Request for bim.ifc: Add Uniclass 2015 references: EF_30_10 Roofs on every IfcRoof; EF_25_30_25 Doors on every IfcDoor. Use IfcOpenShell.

First a look at what the model holds.

```python
import ifcopenshell

model = ifcopenshell.open("bim.ifc")
print(model.schema)
print("classifications:", [c.Name for c in model.by_type("IfcClassification")])
for ifc_class in ("IfcDoor", "IfcRoof", "IfcStair", "IfcWall", "IfcWindow"):
    print(ifc_class, len(model.by_type(ifc_class)))
```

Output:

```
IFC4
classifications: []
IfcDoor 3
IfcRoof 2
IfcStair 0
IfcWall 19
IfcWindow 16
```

```python
import ifcopenshell
import ifcopenshell.api.classification

model = ifcopenshell.open("bim.ifc")

system = ifcopenshell.api.classification.add_classification(model, classification="Uniclass 2015")

codes = {
    "IfcRoof": ("EF_30_10", "Roofs"),
    "IfcDoor": ("EF_25_30_25", "Doors"),
}
for ifc_class, (code, name) in codes.items():
    products = model.by_type(ifc_class)
    ifcopenshell.api.classification.add_reference(
        model, products=products, classification=system, identification=code, name=name
    )
    print(code, len(products))

model.write("bim_updated.ifc")
```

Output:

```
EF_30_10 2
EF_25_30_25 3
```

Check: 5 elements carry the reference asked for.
